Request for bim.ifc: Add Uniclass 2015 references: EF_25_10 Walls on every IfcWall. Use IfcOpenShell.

First a look at what the model holds.

```python
import ifcopenshell

model = ifcopenshell.open("bim.ifc")
print(model.schema)
print("classifications:", [c.Name for c in model.by_type("IfcClassification")])
for ifc_class in ("IfcDoor", "IfcRoof", "IfcStair", "IfcWall", "IfcWindow"):
    print(ifc_class, len(model.by_type(ifc_class)))
```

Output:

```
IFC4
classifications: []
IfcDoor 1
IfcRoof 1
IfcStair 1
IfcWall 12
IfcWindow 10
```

```python
import ifcopenshell
import ifcopenshell.api.classification

model = ifcopenshell.open("bim.ifc")

system = ifcopenshell.api.classification.add_classification(model, classification="Uniclass 2015")

codes = {
    "IfcWall": ("EF_25_10", "Walls"),
}
for ifc_class, (code, name) in codes.items():
    products = model.by_type(ifc_class)
    ifcopenshell.api.classification.add_reference(
        model, products=products, classification=system, identification=code, name=name
    )
    print(code, len(products))

model.write("bim_updated.ifc")
```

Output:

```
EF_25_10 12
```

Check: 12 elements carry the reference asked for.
